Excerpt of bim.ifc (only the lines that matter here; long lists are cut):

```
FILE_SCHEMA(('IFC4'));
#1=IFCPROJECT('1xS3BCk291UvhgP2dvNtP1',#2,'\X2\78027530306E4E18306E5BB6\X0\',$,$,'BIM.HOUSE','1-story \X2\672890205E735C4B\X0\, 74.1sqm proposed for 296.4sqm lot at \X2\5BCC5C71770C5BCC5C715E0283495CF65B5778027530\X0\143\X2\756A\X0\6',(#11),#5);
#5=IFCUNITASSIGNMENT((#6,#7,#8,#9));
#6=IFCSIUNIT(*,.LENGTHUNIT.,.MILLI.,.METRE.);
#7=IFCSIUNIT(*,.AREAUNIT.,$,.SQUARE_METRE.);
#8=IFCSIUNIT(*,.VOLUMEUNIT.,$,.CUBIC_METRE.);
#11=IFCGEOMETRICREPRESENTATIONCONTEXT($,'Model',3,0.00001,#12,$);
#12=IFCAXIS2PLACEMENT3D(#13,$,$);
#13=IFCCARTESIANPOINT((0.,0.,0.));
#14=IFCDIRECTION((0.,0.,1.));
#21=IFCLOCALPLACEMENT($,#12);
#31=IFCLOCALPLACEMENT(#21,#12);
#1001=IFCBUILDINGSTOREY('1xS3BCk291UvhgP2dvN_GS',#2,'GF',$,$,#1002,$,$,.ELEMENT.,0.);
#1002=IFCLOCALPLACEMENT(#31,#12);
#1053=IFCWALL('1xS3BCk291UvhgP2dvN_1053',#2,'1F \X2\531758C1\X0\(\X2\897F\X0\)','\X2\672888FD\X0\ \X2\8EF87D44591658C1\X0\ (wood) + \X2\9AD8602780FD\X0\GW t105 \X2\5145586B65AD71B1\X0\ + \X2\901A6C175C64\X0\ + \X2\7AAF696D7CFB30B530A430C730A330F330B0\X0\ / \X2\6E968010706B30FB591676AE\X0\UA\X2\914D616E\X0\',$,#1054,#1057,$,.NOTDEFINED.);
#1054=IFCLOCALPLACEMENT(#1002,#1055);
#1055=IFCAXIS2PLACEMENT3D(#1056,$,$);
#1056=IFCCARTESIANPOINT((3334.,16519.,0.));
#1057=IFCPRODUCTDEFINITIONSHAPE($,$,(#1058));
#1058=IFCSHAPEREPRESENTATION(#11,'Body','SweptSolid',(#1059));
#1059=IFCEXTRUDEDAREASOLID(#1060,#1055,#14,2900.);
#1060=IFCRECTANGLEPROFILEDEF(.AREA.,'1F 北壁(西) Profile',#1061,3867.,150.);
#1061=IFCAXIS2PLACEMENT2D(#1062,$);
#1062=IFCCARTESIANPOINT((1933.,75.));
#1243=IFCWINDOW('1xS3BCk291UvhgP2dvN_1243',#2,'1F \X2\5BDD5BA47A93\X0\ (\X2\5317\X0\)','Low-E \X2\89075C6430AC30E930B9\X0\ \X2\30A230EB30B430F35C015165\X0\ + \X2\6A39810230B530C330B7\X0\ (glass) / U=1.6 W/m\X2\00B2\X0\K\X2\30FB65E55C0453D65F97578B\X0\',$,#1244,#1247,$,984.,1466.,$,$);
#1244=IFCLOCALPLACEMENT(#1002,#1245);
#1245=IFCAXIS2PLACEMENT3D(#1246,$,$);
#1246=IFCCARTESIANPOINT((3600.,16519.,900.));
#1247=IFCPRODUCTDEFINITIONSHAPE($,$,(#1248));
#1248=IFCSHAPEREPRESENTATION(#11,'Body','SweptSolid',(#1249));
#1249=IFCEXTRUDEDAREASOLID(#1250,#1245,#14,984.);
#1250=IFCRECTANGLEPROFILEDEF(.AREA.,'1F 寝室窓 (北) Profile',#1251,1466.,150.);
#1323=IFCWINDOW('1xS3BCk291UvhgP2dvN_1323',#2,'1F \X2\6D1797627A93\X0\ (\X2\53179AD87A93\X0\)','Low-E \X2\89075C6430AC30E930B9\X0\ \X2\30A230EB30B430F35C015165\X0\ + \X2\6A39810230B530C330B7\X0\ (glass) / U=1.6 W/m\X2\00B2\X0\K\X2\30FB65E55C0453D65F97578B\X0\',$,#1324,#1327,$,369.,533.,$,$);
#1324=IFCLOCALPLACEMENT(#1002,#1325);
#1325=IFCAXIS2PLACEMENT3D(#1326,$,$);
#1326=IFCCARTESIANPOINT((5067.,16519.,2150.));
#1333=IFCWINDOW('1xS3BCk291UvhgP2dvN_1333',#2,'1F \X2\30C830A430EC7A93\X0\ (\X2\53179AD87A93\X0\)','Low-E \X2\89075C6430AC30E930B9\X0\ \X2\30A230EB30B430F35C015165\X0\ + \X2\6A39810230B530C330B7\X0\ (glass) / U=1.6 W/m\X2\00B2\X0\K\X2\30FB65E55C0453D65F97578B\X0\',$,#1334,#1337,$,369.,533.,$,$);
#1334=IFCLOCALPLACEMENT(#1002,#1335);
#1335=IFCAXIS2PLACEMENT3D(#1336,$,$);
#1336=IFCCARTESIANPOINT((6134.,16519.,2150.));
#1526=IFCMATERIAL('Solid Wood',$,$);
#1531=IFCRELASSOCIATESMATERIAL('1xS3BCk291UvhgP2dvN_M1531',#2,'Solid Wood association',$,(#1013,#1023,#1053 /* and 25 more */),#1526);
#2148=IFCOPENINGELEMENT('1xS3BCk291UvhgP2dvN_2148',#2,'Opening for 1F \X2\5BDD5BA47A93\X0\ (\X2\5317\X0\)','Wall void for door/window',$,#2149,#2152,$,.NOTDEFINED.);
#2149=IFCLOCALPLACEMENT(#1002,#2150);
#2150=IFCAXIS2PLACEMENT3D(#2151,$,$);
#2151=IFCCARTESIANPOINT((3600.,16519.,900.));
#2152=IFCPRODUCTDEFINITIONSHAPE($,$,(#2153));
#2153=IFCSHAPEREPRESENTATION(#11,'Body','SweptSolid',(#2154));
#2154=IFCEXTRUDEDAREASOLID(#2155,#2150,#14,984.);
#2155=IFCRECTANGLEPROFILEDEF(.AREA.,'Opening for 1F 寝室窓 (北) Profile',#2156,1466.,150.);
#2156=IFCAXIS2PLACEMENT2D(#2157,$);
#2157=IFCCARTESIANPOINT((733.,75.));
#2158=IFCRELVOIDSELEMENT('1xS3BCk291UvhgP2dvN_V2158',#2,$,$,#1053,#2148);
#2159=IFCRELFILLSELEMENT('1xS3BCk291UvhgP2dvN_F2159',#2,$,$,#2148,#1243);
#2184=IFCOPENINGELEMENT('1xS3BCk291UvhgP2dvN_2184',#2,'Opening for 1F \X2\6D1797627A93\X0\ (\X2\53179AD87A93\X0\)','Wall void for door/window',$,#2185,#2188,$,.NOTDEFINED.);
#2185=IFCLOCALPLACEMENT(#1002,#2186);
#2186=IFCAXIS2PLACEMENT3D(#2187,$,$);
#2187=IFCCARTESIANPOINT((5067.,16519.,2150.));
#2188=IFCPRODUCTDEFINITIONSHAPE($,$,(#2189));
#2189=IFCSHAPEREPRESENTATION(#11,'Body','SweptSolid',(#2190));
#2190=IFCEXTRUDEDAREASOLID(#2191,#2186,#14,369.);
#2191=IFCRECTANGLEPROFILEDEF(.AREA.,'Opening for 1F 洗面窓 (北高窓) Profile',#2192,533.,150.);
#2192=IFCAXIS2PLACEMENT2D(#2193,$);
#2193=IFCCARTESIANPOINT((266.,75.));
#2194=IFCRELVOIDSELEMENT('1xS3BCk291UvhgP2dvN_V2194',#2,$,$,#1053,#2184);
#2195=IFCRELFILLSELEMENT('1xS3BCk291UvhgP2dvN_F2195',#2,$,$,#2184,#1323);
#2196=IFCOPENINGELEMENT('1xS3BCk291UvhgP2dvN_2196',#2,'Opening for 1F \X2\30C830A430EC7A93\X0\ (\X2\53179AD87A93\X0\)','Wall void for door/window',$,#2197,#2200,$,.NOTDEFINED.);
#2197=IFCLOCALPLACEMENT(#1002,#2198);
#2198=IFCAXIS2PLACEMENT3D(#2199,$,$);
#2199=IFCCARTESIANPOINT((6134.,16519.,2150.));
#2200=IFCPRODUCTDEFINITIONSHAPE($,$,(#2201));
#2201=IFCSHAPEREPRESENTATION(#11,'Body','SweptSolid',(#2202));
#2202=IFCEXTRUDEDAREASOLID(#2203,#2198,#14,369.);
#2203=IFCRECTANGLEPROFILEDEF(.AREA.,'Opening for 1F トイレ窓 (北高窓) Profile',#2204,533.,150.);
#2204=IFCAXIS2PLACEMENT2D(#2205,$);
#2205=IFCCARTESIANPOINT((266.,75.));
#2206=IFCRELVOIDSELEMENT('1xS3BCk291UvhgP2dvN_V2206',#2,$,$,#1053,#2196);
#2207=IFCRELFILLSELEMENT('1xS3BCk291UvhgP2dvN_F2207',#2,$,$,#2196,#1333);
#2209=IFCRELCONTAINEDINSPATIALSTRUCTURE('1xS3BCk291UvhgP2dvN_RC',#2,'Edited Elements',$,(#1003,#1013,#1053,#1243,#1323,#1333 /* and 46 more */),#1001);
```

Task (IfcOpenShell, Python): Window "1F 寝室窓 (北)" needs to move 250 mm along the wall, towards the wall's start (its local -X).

```python
import ifcopenshell
import ifcopenshell.api.geometry
import ifcopenshell.util.placement
import ifcopenshell.util.unit

model = ifcopenshell.open("bim.ifc")
unit_scale = ifcopenshell.util.unit.calculate_unit_scale(model)

window = model.by_id(1243)
opening = window.FillsVoids[0].RelatingOpeningElement
wall = opening.VoidsElements[0].RelatingBuildingElement

wall_matrix = ifcopenshell.util.placement.get_local_placement(wall.ObjectPlacement)
shift = wall_matrix[:3, 0] * -0.25 / unit_scale
before = ifcopenshell.util.placement.get_local_placement(window.ObjectPlacement)[:3, 3].copy()

# The window is not placed relative to its opening, so move both.
for product in (opening, window):
    matrix = ifcopenshell.util.placement.get_local_placement(product.ObjectPlacement)
    matrix[:3, 3] += shift
    ifcopenshell.api.geometry.edit_object_placement(model, product=product, matrix=matrix, is_si=False)

after = ifcopenshell.util.placement.get_local_placement(window.ObjectPlacement)[:3, 3]
print("window moved by", (after - before).round(3) + 0.0)

model.write("bim_rev.ifc")
```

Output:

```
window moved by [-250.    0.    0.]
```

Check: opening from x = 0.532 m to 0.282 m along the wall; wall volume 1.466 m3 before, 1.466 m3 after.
